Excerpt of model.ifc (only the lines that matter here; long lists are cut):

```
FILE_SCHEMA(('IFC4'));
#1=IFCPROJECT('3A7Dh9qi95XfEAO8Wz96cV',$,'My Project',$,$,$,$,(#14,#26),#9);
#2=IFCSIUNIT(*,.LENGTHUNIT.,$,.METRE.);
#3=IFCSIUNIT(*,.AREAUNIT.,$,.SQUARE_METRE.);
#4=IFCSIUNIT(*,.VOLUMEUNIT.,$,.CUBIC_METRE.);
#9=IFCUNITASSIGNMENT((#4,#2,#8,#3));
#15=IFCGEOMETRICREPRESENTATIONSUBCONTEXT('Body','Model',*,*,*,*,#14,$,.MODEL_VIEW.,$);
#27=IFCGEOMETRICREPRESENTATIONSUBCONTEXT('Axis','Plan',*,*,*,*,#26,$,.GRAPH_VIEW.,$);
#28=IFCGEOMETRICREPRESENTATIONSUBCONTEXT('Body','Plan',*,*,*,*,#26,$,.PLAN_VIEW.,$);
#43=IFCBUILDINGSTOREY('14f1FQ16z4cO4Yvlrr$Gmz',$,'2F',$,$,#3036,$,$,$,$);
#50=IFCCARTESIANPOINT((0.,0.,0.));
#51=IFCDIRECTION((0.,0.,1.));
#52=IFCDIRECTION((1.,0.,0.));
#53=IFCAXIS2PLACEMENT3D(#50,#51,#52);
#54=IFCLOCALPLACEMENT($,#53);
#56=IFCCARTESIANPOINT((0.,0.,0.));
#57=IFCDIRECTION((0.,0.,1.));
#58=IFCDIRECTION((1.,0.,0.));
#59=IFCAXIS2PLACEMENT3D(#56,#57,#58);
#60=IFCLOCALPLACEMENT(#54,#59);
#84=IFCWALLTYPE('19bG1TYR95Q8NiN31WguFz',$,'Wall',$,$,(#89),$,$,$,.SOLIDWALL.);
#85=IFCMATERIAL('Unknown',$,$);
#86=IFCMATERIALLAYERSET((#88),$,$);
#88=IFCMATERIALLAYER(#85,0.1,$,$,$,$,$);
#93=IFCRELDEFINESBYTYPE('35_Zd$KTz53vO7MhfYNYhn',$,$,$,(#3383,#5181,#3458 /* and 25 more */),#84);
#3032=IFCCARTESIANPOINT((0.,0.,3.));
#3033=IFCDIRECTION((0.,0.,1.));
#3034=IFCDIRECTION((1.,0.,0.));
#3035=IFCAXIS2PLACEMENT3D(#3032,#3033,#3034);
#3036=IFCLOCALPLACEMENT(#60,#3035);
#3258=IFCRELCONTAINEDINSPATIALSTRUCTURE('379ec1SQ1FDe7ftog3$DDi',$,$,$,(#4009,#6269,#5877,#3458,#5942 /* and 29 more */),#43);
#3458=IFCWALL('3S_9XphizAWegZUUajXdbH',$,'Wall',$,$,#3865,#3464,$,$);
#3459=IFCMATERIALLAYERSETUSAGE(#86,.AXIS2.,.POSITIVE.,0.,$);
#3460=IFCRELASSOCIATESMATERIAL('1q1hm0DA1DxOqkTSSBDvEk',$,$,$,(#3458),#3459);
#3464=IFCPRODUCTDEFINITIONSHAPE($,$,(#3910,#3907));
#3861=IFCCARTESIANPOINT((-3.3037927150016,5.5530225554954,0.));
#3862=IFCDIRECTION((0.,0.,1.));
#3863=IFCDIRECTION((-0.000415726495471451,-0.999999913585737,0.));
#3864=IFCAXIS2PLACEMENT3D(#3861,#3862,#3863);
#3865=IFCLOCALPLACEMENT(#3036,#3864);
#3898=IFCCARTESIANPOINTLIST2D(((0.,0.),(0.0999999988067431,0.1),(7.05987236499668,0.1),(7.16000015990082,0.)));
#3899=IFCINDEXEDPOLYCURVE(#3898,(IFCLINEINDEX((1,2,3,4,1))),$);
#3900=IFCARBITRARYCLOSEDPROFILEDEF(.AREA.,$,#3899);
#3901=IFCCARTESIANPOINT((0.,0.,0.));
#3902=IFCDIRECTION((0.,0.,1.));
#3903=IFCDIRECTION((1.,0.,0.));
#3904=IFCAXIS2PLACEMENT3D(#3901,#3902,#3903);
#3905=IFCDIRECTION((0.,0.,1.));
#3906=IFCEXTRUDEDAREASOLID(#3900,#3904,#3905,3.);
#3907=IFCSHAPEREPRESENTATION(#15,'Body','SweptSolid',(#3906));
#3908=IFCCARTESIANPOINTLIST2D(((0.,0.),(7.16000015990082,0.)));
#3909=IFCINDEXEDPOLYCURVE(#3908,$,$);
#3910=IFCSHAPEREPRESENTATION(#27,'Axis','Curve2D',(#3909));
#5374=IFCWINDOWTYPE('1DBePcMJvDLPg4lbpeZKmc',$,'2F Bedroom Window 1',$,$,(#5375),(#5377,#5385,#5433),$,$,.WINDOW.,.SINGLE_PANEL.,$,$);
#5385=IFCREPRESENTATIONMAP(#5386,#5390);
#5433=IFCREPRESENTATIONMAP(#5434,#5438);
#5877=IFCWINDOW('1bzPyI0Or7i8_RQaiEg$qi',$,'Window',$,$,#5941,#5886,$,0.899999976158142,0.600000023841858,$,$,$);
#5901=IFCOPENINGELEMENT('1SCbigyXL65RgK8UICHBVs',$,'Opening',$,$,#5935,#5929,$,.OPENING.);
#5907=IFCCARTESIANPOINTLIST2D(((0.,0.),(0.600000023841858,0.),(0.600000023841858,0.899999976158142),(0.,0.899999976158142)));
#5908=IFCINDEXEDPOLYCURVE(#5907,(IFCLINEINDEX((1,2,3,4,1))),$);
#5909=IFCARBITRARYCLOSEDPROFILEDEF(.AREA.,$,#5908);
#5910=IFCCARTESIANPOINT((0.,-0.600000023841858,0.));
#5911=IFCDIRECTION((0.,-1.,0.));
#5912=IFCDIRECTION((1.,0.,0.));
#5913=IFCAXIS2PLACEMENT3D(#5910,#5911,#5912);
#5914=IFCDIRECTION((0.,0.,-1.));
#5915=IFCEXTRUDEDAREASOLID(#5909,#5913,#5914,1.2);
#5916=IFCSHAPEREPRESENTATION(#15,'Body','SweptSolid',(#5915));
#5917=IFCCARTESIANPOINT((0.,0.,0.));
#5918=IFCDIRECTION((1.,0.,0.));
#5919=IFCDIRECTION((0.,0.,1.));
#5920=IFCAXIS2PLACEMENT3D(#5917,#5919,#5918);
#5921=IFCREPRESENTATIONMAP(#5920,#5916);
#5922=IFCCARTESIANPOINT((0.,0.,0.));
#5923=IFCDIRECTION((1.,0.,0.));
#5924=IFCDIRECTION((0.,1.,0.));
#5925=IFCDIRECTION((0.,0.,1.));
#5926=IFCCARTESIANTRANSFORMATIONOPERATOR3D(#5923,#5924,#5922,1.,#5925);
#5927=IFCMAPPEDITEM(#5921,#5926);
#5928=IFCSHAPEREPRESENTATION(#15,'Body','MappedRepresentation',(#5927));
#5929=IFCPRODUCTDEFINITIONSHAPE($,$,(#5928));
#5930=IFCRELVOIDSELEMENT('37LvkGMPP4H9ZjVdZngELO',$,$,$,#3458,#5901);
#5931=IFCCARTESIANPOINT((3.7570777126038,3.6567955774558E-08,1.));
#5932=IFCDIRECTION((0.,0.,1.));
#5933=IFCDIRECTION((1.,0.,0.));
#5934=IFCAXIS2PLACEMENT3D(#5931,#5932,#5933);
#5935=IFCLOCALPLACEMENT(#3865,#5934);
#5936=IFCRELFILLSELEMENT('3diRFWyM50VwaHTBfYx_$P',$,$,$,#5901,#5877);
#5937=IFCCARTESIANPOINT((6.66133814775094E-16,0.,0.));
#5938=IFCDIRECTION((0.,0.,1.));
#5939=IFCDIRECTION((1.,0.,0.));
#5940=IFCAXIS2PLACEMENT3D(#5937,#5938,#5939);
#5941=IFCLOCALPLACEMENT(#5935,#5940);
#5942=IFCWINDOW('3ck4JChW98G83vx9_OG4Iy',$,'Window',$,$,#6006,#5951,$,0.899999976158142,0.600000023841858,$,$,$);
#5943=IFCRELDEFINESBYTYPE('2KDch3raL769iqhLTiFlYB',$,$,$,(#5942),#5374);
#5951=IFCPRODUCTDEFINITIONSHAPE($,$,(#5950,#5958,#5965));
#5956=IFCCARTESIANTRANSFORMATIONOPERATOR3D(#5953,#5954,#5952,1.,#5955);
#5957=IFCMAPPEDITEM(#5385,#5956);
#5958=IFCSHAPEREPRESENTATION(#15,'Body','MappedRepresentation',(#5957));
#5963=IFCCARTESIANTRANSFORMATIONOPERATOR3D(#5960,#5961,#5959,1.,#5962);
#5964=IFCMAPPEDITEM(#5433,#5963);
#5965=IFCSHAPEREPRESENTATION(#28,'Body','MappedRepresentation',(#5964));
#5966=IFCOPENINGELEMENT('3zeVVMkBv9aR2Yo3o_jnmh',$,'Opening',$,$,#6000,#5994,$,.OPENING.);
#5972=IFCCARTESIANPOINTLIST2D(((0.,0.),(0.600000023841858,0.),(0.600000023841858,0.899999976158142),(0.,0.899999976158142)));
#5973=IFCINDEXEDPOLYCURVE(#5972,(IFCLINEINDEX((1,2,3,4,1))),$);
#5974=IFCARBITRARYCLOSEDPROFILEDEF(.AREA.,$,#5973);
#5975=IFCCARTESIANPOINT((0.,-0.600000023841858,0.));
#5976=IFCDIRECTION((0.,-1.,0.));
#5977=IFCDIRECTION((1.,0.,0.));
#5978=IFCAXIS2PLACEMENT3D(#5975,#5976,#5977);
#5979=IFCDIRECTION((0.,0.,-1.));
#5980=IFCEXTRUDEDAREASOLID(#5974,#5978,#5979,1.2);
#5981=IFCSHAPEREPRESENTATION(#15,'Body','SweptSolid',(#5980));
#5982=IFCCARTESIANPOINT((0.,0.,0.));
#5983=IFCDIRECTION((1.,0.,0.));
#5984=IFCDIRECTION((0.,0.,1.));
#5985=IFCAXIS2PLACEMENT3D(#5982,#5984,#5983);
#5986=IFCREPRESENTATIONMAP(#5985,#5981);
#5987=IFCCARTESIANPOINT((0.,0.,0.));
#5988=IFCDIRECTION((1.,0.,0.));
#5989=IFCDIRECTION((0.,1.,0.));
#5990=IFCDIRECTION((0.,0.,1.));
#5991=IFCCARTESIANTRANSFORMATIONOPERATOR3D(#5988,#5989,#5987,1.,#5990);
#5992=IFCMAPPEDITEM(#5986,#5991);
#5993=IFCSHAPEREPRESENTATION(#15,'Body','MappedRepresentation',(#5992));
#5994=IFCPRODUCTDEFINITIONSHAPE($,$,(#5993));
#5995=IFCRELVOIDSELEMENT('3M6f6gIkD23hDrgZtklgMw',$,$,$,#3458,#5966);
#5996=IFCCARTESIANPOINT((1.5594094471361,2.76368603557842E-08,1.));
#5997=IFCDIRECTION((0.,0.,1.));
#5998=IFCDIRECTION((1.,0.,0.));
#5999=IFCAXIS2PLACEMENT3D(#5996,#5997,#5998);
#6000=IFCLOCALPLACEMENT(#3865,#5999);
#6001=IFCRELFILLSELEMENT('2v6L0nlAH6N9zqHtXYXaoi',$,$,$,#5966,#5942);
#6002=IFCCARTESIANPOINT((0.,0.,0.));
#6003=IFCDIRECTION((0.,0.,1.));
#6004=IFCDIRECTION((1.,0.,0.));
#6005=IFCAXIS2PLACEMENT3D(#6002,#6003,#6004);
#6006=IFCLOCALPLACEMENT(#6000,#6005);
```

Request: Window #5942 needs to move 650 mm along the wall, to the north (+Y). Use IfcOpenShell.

```python
import ifcopenshell
import ifcopenshell.api.geometry
import ifcopenshell.util.placement
import ifcopenshell.util.unit

model = ifcopenshell.open("model.ifc")
unit_scale = ifcopenshell.util.unit.calculate_unit_scale(model)

window = model.by_guid("3ck4JChW98G83vx9_OG4Iy")
opening = window.FillsVoids[0].RelatingOpeningElement
wall = opening.VoidsElements[0].RelatingBuildingElement

wall_matrix = ifcopenshell.util.placement.get_local_placement(wall.ObjectPlacement)
shift = wall_matrix[:3, 0] * -0.65 / unit_scale
before = ifcopenshell.util.placement.get_local_placement(window.ObjectPlacement)[:3, 3].copy()

# The window is placed relative to its opening, so it follows when the opening moves.
matrix = ifcopenshell.util.placement.get_local_placement(opening.ObjectPlacement)
matrix[:3, 3] += shift
ifcopenshell.api.geometry.edit_object_placement(
    model, product=opening, matrix=matrix, is_si=False, should_transform_children=True
)

after = ifcopenshell.util.placement.get_local_placement(window.ObjectPlacement)[:3, 3]
print("window moved by", (after - before).round(3) + 0.0)

model.write("model_updated.ifc")
```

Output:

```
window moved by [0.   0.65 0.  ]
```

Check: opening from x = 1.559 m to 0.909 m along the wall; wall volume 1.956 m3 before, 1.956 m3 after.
